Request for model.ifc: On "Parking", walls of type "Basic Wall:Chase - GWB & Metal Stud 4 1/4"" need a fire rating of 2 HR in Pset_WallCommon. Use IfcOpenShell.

First a look at what the model holds.

```python
import ifcopenshell
import ifcopenshell.util.element

model = ifcopenshell.open("model.ifc")
print(model.schema)
storey = next(s for s in model.by_type("IfcBuildingStorey") if s.Name == "Parking")
walls = [e for e in ifcopenshell.util.element.get_decomposition(storey) if e.is_a("IfcWall")]
seen = {}
for e in walls:
    element_type = ifcopenshell.util.element.get_type(e)
    key = (element_type.Name if element_type != e and element_type else None, ifcopenshell.util.element.get_pset(e, "Pset_WallCommon", "FireRating"))
    seen[key] = seen.get(key, 0) + 1
for (name, value), count in sorted(seen.items(), key=str):
    print(count, "x", name, "|", value)
```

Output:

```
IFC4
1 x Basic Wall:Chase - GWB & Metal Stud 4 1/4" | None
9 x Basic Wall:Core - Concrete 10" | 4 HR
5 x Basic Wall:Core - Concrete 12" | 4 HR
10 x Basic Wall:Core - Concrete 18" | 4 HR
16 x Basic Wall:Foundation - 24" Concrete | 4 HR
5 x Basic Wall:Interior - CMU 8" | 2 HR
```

```python
import ifcopenshell
import ifcopenshell.api.pset
import ifcopenshell.util.element

model = ifcopenshell.open("model.ifc")

storey = next(s for s in model.by_type("IfcBuildingStorey") if s.Name == "Parking")
walls = [e for e in ifcopenshell.util.element.get_decomposition(storey) if e.is_a("IfcWall")]

count = 0
for e in walls:
    element_type = ifcopenshell.util.element.get_type(e)
    if element_type in (None, e) or element_type.Name != 'Basic Wall:Chase - GWB & Metal Stud 4 1/4"':
        continue
    # add_pset returns the element's existing set when there is one.
    pset = ifcopenshell.api.pset.add_pset(model, product=e, name="Pset_WallCommon")
    ifcopenshell.api.pset.edit_pset(model, pset=pset, properties={"FireRating": "2 HR"})
    count += 1

print(count, "walls updated")

model.write("model_updated.ifc")
```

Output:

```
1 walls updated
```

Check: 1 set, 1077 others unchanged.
